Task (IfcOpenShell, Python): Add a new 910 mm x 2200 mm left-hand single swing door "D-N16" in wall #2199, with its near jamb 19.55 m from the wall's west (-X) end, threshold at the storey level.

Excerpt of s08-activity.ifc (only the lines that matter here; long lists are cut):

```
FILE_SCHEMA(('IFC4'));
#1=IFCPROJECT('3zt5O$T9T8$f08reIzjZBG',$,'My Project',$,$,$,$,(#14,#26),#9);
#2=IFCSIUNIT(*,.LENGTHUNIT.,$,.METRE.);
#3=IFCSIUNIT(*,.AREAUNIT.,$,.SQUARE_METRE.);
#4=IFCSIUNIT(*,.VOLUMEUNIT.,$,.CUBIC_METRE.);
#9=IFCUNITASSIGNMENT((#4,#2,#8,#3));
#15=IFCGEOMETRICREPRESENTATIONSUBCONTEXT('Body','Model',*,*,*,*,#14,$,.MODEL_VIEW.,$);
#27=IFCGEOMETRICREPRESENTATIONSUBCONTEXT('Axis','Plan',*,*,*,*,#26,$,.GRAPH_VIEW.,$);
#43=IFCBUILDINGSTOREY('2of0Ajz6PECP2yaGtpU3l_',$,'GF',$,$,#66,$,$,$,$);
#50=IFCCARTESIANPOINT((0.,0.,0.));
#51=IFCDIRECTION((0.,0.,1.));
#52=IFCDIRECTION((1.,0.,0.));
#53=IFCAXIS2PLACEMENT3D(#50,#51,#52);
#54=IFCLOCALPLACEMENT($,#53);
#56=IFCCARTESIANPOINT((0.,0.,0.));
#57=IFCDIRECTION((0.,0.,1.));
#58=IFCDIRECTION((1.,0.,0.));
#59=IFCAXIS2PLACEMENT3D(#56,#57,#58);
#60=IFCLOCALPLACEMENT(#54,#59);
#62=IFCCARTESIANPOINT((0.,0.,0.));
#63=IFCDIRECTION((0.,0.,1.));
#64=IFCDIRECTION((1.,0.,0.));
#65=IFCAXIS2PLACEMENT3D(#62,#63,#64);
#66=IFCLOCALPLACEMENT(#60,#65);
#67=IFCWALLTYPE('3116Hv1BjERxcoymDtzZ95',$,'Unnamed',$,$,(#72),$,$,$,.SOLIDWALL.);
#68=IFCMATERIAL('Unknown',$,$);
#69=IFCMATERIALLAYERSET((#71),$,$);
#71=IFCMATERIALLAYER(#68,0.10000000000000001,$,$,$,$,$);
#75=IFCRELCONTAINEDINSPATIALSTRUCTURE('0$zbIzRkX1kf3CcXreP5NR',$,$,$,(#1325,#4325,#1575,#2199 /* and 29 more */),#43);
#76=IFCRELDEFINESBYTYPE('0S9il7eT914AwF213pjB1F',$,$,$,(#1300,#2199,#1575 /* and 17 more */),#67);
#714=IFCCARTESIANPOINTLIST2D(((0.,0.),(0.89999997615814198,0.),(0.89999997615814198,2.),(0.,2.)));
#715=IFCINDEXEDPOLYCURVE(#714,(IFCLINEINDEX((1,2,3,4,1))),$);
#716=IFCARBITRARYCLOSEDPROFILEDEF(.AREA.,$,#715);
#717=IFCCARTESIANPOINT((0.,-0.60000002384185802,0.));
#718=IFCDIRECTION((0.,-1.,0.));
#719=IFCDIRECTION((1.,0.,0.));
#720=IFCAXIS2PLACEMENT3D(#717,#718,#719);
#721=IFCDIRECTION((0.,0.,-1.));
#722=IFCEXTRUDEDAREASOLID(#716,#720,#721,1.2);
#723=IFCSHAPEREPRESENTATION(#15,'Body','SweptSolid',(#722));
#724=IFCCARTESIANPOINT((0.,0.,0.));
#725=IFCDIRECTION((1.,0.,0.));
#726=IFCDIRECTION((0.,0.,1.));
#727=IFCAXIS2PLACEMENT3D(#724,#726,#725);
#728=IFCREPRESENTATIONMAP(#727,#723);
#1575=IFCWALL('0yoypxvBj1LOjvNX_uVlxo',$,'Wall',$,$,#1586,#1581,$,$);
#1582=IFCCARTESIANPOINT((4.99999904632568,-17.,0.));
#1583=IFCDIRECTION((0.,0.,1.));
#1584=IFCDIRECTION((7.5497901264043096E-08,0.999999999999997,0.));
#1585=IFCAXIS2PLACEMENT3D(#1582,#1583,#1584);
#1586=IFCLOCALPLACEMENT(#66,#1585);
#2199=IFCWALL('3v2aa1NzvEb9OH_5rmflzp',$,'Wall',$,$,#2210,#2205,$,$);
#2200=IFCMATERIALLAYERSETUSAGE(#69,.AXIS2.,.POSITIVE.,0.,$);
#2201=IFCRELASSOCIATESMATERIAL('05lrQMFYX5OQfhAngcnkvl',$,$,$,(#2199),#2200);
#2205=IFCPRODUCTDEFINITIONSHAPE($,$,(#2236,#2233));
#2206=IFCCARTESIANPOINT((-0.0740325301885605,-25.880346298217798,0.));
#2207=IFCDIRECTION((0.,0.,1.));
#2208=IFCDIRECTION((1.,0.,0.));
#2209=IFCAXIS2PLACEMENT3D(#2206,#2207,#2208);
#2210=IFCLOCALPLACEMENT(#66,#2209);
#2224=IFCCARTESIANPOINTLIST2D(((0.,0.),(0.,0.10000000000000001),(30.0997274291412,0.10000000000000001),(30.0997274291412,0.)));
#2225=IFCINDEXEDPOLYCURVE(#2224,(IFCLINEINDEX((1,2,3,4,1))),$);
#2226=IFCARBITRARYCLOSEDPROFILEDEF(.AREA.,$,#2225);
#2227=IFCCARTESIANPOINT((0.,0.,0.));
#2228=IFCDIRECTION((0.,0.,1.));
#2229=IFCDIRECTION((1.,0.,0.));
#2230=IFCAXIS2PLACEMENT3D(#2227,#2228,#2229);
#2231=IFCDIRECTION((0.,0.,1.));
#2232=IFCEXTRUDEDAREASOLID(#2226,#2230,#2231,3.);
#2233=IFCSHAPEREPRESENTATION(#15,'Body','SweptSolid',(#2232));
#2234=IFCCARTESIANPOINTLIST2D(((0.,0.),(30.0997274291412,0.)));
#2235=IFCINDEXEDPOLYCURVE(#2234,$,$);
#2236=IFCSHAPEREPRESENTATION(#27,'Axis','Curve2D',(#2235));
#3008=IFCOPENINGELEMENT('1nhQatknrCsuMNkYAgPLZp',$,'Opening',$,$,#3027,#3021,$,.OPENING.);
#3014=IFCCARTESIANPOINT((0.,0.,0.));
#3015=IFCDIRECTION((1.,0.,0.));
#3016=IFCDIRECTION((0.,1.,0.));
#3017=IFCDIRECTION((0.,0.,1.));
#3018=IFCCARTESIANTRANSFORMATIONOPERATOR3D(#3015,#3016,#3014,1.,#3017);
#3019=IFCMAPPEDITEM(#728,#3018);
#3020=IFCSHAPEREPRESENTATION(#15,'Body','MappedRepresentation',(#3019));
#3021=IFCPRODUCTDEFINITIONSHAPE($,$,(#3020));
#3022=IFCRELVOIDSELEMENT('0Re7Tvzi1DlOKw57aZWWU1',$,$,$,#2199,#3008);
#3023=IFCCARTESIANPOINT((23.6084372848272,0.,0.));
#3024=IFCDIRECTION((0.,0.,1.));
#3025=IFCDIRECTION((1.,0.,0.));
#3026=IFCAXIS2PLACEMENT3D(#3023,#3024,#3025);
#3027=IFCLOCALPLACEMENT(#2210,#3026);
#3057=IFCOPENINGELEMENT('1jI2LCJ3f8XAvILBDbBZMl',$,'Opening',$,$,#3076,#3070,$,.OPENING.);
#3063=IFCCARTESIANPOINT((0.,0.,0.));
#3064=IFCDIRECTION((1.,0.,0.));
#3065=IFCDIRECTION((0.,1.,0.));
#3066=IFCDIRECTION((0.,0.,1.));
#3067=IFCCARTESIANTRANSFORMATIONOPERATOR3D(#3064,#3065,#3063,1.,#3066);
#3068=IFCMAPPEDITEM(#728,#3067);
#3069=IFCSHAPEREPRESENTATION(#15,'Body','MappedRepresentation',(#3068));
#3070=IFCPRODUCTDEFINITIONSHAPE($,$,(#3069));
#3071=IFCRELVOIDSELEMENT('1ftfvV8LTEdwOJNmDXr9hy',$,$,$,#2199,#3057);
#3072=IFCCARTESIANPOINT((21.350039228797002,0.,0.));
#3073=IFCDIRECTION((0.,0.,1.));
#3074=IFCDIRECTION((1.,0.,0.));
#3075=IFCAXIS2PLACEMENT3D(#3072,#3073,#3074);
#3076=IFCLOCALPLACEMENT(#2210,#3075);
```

```python
import numpy as np
import ifcopenshell
import ifcopenshell.api.feature
import ifcopenshell.api.geometry
import ifcopenshell.api.root
import ifcopenshell.api.spatial
import ifcopenshell.geom
import ifcopenshell.util.element
import ifcopenshell.util.placement
import ifcopenshell.util.representation
import ifcopenshell.util.shape
import ifcopenshell.util.unit

model = ifcopenshell.open("s08-activity.ifc")
unit_scale = ifcopenshell.util.unit.calculate_unit_scale(model)
settings = ifcopenshell.geom.settings()


def volume(element):
    """Net volume in cubic metres, openings subtracted."""
    shape = ifcopenshell.geom.create_shape(settings, element)
    return ifcopenshell.util.shape.get_volume(shape.geometry)


wall = model.by_id(2199)
storey = ifcopenshell.util.element.get_container(wall, ifc_class="IfcBuildingStorey")
context = ifcopenshell.util.representation.get_context(model, "Model", "Body", "MODEL_VIEW")
before = volume(wall)

width, height, from_end, sill = 0.91, 2.2, 19.55, 0.0  # metres

# The wall runs along its own X axis, and the end named is its -X end.
wall_shape = ifcopenshell.geom.create_shape(settings, wall)
x, y, z = ifcopenshell.util.shape.get_vertices(wall_shape.geometry).T
start = x.min() + from_end
face, thickness = float(y.min()), float(y.max() - y.min())
wall_matrix = ifcopenshell.util.placement.get_local_placement(wall.ObjectPlacement)
level = ifcopenshell.util.placement.get_local_placement(storey.ObjectPlacement)[2, 3]


def in_wall(x, y):
    """Placement at x, y metres in the wall's axes, at sill height."""
    matrix = wall_matrix.copy()
    matrix[:, 3] = wall_matrix @ np.array([x / unit_scale, y / unit_scale, 0.0, 1.0])
    matrix[2, 3] = level + sill / unit_scale
    return matrix


# Opening: a box that overshoots both wall faces by 50 mm.
opening = ifcopenshell.api.root.create_entity(model, ifc_class="IfcOpeningElement", predefined_type="OPENING")
box = ifcopenshell.api.geometry.add_wall_representation(
    model, context=context, length=width, height=height, thickness=thickness + 0.1
)
ifcopenshell.api.geometry.assign_representation(model, product=opening, representation=box)
ifcopenshell.api.geometry.edit_object_placement(model, product=opening, matrix=in_wall(start, face - 0.05), is_si=False)
ifcopenshell.api.feature.add_feature(model, feature=opening, element=wall)

door = ifcopenshell.api.root.create_entity(model, ifc_class="IfcDoor", name="D-N16", predefined_type="DOOR")
door.OverallWidth, door.OverallHeight = width / unit_scale, height / unit_scale
door.OperationType = "SINGLE_SWING_LEFT"
body = ifcopenshell.api.geometry.add_door_representation(
    model,
    context=context,
    overall_width=door.OverallWidth,
    overall_height=door.OverallHeight,
    operation_type="SINGLE_SWING_LEFT",
    lining_properties={"LiningDepth": thickness / unit_scale, "ThresholdDepth": thickness / unit_scale},
)
ifcopenshell.api.geometry.assign_representation(model, product=door, representation=body)
ifcopenshell.api.spatial.assign_container(model, products=[door], relating_structure=storey)
ifcopenshell.api.feature.add_filling(model, opening=opening, element=door)

# The lining spans the wall, so the door starts at the wall face.
ifcopenshell.api.geometry.edit_object_placement(model, product=door, matrix=in_wall(start, face), is_si=False)

after = volume(wall)

print(f"wall volume {before:.3f} -> {after:.3f} m3")

model.write("s08-activity_updated.ifc")
```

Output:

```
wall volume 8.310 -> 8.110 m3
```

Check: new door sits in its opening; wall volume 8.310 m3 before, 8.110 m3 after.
